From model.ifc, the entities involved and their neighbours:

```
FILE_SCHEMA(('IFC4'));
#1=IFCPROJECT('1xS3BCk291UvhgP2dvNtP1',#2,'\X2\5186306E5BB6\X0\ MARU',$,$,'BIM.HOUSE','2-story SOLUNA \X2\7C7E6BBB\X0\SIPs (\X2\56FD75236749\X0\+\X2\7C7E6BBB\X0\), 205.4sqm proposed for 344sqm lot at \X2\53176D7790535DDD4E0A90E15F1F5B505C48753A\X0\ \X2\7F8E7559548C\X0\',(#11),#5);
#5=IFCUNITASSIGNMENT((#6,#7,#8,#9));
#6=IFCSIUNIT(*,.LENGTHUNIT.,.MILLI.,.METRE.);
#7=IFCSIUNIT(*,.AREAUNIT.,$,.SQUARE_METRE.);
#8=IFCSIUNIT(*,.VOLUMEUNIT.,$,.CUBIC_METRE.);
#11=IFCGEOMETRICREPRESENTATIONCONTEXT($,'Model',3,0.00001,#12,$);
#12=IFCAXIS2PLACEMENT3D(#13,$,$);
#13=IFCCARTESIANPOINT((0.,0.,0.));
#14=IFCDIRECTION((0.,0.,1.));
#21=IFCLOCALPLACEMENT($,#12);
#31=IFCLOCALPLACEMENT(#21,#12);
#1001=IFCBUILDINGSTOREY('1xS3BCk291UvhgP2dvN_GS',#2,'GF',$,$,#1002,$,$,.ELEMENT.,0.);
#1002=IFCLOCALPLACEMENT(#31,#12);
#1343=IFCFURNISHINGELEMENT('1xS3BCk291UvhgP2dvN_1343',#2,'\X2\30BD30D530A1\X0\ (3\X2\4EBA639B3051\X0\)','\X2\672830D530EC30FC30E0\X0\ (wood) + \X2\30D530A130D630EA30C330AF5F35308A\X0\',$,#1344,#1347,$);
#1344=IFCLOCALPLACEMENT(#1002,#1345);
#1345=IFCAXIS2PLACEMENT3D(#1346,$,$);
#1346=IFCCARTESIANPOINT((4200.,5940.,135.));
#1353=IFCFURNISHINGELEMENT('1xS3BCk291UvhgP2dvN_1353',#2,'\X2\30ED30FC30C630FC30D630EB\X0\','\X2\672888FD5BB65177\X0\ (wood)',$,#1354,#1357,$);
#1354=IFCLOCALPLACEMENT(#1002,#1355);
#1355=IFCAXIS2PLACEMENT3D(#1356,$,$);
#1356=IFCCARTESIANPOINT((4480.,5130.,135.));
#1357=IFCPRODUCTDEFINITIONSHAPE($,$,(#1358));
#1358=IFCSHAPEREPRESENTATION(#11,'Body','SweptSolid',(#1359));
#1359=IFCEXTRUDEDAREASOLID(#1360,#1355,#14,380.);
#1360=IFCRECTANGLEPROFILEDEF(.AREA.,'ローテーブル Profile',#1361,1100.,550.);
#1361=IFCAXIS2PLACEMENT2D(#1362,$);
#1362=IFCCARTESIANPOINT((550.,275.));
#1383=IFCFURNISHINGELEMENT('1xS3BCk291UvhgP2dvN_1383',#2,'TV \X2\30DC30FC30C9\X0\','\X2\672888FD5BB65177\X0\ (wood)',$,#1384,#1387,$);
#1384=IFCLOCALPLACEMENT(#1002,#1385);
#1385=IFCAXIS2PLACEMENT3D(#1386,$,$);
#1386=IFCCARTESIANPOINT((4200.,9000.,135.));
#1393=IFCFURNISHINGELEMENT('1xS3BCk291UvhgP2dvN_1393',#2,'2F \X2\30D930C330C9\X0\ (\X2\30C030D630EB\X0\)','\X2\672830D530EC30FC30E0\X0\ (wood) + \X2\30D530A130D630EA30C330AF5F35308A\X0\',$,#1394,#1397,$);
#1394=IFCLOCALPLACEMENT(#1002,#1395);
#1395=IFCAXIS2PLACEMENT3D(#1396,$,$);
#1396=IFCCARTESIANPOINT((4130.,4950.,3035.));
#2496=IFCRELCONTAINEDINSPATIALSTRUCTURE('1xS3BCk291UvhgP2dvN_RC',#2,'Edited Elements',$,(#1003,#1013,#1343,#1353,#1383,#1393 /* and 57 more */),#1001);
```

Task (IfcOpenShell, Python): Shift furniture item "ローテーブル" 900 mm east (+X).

```python
import ifcopenshell
import ifcopenshell.api.geometry
import ifcopenshell.util.placement
import ifcopenshell.util.unit

model = ifcopenshell.open("model.ifc")
unit_scale = ifcopenshell.util.unit.calculate_unit_scale(model)

item = model.by_guid("1xS3BCk291UvhgP2dvN_1353")
matrix = ifcopenshell.util.placement.get_local_placement(item.ObjectPlacement)
matrix[0, 3] += 0.9 / unit_scale
ifcopenshell.api.geometry.edit_object_placement(model, product=item, matrix=matrix, is_si=False)

print(ifcopenshell.util.placement.get_local_placement(item.ObjectPlacement).round(3) + 0.0)

model.write("model-out.ifc")
```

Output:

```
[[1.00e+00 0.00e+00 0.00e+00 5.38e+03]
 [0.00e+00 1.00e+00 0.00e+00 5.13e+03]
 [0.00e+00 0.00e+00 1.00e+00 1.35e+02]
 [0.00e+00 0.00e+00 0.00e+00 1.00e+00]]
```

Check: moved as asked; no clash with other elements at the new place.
